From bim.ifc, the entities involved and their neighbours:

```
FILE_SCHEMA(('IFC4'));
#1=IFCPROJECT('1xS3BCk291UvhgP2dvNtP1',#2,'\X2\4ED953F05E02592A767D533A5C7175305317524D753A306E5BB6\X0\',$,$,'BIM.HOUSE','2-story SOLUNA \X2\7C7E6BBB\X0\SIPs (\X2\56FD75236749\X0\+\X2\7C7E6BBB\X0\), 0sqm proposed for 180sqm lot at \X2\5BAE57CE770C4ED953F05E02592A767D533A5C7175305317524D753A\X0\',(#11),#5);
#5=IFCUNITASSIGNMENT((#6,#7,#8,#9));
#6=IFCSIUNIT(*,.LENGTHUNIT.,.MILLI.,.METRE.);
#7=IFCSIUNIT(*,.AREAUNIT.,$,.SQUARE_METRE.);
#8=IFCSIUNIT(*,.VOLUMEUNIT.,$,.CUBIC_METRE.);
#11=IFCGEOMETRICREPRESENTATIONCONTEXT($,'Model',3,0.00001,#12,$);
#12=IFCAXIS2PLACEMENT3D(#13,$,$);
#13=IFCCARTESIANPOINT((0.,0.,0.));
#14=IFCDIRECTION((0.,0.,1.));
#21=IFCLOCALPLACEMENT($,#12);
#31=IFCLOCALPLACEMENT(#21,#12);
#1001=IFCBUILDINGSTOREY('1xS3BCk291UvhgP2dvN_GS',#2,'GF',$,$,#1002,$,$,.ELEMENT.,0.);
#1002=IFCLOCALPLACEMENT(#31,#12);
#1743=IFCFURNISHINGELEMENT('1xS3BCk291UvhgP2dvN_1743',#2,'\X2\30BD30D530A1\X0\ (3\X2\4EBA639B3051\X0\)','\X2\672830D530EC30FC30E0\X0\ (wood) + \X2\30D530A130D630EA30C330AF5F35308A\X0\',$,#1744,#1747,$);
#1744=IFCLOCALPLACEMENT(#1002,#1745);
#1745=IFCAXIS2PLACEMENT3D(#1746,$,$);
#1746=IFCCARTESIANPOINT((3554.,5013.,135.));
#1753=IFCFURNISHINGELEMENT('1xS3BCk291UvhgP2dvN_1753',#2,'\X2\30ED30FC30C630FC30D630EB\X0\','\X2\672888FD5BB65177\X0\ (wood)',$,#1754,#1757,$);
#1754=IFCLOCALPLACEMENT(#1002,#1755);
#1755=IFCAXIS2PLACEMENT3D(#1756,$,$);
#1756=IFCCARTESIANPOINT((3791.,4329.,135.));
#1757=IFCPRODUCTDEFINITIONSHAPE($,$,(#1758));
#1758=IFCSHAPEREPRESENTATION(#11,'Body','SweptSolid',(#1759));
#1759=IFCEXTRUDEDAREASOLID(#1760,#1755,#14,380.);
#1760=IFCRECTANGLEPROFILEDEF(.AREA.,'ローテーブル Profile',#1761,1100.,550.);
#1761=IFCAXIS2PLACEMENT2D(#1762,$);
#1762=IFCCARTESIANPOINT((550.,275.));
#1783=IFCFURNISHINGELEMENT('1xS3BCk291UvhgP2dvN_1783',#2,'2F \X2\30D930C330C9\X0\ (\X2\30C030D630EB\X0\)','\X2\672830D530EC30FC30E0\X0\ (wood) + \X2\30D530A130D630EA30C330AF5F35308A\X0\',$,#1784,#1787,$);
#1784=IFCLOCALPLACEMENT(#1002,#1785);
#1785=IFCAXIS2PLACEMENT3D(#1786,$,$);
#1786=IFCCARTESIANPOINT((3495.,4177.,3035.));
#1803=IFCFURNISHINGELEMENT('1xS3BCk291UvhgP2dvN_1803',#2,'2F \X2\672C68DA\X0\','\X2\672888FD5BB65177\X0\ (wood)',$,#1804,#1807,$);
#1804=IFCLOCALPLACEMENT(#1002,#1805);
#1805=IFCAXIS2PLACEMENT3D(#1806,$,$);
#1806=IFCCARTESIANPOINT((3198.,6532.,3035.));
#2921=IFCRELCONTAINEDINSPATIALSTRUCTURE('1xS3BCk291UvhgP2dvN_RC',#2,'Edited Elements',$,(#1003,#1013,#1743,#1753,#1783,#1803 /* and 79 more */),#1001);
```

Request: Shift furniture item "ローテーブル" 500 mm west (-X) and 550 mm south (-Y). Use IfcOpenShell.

```python
import ifcopenshell
import ifcopenshell.api.geometry
import ifcopenshell.util.placement

model = ifcopenshell.open("bim.ifc")

item = model.by_guid("1xS3BCk291UvhgP2dvN_1753")
matrix = ifcopenshell.util.placement.get_local_placement(item.ObjectPlacement)
matrix[0, 3] -= 500.0
matrix[1, 3] -= 550.0
ifcopenshell.api.geometry.edit_object_placement(model, product=item, matrix=matrix, is_si=False)

print(ifcopenshell.util.placement.get_local_placement(item.ObjectPlacement).round(3) + 0.0)

model.write("bim_v2.ifc")
```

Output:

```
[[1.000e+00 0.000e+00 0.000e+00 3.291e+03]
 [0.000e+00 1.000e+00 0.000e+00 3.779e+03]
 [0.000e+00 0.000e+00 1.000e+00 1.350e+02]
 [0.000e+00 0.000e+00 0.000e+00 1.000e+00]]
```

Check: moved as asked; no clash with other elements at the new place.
